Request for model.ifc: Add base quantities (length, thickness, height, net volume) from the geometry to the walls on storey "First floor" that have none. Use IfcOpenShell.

First a look at what the model holds.

```python
import ifcopenshell
import ifcopenshell.util.element
import ifcopenshell.util.unit

model = ifcopenshell.open("model.ifc")
print(model.schema)
for unit_type in ("LENGTHUNIT", "AREAUNIT", "VOLUMEUNIT"):
    print(unit_type, ifcopenshell.util.unit.calculate_unit_scale(model, unit_type))
storey = next(s for s in model.by_type("IfcBuildingStorey") if s.Name == "First floor")
walls = [e for e in ifcopenshell.util.element.get_decomposition(storey) if e.is_a("IfcWall")]
for e in sorted(walls, key=lambda e: e.id()):
    print(e.id(), e.is_a(), e.Name, list(ifcopenshell.util.element.get_psets(e, qtos_only=True)), sep=" | ")
```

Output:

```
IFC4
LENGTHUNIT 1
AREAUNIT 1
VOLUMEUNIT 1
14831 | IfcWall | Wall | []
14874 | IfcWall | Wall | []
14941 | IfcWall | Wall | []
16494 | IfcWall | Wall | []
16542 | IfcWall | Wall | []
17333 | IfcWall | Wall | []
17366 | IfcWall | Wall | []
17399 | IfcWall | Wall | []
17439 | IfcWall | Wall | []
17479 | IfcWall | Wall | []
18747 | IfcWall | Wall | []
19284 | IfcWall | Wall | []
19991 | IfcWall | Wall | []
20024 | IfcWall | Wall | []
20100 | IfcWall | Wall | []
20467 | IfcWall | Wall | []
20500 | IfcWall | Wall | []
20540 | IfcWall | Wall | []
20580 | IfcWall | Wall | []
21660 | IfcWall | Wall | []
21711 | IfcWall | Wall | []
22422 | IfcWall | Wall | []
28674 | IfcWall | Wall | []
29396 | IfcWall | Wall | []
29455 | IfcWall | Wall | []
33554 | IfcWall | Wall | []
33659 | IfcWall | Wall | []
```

```python
import ifcopenshell
import ifcopenshell.api.pset
import ifcopenshell.geom
import ifcopenshell.util.element
import ifcopenshell.util.shape
import ifcopenshell.util.unit

model = ifcopenshell.open("model.ifc")
unit_scale = ifcopenshell.util.unit.calculate_unit_scale(model)
volume_scale = ifcopenshell.util.unit.calculate_unit_scale(model, "VOLUMEUNIT")
settings = ifcopenshell.geom.settings()

storey = next(s for s in model.by_type("IfcBuildingStorey") if s.Name == "First floor")
walls = [e for e in ifcopenshell.util.element.get_decomposition(storey) if e.is_a("IfcWall")]

for e in sorted(walls, key=lambda e: e.id()):
    if ifcopenshell.util.element.get_psets(e, qtos_only=True, should_inherit=False):
        continue
    # Geometry comes back in metres, in the element's own axes.
    shape = ifcopenshell.geom.create_shape(settings, e)
    values = {
        "Length": ifcopenshell.util.shape.get_x(shape.geometry) / unit_scale,
        "Width": ifcopenshell.util.shape.get_y(shape.geometry) / unit_scale,
        "Height": ifcopenshell.util.shape.get_z(shape.geometry) / unit_scale,
        "NetVolume": ifcopenshell.util.shape.get_volume(shape.geometry) / volume_scale,
    }
    qto = ifcopenshell.api.pset.add_qto(model, product=e, name="Qto_WallBaseQuantities")
    ifcopenshell.api.pset.edit_qto(model, qto=qto, properties=values)
    print(e.id(), {k: round(v, 3) for k, v in values.items()})

model.write("model_v2.ifc")
```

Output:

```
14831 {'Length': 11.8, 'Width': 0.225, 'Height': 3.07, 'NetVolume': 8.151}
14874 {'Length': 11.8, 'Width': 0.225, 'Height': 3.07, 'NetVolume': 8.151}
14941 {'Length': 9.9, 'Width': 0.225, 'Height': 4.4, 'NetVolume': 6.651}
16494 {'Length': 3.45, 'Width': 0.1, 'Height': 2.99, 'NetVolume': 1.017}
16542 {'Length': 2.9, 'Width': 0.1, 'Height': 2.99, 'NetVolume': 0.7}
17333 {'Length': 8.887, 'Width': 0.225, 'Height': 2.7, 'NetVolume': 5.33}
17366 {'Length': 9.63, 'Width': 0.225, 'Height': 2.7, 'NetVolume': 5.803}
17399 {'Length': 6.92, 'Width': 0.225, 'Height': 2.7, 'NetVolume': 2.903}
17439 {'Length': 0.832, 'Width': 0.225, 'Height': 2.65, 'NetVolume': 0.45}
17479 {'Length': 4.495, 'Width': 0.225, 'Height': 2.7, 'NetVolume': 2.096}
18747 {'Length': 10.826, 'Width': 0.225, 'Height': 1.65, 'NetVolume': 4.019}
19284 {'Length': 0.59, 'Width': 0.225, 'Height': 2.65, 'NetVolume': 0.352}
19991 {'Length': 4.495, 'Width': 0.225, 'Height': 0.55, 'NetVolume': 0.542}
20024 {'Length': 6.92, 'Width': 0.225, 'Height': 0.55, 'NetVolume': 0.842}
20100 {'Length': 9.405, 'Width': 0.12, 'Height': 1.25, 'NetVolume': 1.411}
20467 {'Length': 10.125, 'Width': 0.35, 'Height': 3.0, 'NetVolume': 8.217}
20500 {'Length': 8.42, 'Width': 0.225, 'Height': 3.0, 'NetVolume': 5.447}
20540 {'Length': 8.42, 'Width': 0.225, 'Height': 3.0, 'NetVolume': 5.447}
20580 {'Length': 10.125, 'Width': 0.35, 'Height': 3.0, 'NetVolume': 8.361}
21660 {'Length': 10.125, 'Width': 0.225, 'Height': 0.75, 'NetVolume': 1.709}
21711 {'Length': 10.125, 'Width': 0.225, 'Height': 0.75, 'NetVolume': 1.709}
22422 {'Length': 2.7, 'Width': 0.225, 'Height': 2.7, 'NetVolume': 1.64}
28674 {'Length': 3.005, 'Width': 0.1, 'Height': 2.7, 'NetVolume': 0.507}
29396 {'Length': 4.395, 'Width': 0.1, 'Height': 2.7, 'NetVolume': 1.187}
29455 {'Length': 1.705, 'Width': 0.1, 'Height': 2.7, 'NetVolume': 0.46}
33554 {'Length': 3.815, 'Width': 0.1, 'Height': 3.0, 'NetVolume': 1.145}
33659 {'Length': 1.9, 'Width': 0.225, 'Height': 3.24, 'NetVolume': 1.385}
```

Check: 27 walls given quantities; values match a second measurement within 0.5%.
